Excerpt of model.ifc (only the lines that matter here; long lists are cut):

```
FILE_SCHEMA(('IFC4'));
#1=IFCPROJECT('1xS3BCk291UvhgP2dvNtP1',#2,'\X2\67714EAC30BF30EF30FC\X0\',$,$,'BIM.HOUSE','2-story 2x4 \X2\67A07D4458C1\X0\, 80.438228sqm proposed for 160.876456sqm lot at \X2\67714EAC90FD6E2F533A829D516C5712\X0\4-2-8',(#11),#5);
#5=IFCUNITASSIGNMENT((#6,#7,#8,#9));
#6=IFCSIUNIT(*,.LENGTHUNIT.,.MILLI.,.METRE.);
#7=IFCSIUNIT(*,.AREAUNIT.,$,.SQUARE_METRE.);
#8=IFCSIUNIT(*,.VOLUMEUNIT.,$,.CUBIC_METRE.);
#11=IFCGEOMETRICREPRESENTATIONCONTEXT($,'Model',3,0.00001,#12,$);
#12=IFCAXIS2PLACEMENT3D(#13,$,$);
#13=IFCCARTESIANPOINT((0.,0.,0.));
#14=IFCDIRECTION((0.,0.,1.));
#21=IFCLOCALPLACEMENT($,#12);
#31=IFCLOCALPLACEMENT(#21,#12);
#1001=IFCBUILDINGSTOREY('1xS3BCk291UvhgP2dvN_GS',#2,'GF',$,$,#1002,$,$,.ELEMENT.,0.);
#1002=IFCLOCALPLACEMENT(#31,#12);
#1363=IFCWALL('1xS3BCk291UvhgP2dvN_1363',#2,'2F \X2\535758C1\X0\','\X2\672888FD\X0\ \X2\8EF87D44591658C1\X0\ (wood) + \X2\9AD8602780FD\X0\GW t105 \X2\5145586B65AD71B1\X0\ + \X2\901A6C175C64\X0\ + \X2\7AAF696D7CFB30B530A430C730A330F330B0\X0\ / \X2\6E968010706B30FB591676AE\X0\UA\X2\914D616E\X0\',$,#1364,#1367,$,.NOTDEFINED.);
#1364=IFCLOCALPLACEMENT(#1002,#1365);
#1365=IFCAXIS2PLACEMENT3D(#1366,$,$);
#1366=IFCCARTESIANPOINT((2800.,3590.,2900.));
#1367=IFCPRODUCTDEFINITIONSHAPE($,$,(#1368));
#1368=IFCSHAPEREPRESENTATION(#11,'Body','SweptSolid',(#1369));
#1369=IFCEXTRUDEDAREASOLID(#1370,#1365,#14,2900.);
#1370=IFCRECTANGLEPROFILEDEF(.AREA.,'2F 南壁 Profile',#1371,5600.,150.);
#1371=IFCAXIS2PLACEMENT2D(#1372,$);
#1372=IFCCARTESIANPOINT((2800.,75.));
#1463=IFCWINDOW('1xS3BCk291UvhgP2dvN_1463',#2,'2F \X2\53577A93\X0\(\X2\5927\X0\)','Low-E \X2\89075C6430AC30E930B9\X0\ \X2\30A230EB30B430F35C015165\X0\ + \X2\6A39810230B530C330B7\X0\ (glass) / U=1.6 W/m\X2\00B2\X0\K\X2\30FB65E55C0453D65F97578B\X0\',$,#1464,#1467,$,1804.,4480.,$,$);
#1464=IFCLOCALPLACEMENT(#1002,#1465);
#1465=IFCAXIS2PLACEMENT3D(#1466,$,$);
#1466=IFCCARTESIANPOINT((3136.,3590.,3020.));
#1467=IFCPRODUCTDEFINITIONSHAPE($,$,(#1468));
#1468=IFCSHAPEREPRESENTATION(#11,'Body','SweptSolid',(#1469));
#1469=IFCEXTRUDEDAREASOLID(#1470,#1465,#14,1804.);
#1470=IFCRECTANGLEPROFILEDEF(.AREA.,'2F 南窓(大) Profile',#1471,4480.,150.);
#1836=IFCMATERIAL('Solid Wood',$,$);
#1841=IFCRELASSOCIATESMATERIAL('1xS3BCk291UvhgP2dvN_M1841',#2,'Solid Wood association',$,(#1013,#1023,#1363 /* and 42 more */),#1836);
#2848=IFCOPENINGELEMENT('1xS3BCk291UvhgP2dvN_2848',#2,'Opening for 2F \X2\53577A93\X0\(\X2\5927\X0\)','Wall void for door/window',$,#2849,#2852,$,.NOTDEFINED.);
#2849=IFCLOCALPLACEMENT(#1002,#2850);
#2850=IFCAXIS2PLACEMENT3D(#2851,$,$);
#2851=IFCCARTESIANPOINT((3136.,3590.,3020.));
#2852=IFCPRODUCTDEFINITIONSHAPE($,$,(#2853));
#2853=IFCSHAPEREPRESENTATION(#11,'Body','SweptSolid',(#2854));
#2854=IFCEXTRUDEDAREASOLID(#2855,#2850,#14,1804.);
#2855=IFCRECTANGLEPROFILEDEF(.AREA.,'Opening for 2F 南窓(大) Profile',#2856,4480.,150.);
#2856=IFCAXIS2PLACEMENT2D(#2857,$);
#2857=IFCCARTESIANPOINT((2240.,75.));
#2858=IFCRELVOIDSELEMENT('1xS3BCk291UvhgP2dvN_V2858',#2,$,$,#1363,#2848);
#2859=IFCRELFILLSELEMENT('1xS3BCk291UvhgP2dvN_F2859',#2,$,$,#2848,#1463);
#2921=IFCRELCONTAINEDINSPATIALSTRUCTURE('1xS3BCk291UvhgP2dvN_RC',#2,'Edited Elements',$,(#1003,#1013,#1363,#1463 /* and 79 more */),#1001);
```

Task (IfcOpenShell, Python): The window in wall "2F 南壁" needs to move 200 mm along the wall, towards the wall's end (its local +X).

```python
import ifcopenshell
import ifcopenshell.api.geometry
import ifcopenshell.util.placement
import ifcopenshell.util.unit

model = ifcopenshell.open("model.ifc")
unit_scale = ifcopenshell.util.unit.calculate_unit_scale(model)

window = model.by_guid("1xS3BCk291UvhgP2dvN_1463")
opening = window.FillsVoids[0].RelatingOpeningElement
wall = opening.VoidsElements[0].RelatingBuildingElement

wall_matrix = ifcopenshell.util.placement.get_local_placement(wall.ObjectPlacement)
shift = wall_matrix[:3, 0] * 0.2 / unit_scale
before = ifcopenshell.util.placement.get_local_placement(window.ObjectPlacement)[:3, 3].copy()

# The window is not placed relative to its opening, so move both.
for product in (opening, window):
    matrix = ifcopenshell.util.placement.get_local_placement(product.ObjectPlacement)
    matrix[:3, 3] += shift
    ifcopenshell.api.geometry.edit_object_placement(model, product=product, matrix=matrix, is_si=False)

after = ifcopenshell.util.placement.get_local_placement(window.ObjectPlacement)[:3, 3]
print("window moved by", (after - before).round(3) + 0.0)

model.write("model_updated.ifc")
```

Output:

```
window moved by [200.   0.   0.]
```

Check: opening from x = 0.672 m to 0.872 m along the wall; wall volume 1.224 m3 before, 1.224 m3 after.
